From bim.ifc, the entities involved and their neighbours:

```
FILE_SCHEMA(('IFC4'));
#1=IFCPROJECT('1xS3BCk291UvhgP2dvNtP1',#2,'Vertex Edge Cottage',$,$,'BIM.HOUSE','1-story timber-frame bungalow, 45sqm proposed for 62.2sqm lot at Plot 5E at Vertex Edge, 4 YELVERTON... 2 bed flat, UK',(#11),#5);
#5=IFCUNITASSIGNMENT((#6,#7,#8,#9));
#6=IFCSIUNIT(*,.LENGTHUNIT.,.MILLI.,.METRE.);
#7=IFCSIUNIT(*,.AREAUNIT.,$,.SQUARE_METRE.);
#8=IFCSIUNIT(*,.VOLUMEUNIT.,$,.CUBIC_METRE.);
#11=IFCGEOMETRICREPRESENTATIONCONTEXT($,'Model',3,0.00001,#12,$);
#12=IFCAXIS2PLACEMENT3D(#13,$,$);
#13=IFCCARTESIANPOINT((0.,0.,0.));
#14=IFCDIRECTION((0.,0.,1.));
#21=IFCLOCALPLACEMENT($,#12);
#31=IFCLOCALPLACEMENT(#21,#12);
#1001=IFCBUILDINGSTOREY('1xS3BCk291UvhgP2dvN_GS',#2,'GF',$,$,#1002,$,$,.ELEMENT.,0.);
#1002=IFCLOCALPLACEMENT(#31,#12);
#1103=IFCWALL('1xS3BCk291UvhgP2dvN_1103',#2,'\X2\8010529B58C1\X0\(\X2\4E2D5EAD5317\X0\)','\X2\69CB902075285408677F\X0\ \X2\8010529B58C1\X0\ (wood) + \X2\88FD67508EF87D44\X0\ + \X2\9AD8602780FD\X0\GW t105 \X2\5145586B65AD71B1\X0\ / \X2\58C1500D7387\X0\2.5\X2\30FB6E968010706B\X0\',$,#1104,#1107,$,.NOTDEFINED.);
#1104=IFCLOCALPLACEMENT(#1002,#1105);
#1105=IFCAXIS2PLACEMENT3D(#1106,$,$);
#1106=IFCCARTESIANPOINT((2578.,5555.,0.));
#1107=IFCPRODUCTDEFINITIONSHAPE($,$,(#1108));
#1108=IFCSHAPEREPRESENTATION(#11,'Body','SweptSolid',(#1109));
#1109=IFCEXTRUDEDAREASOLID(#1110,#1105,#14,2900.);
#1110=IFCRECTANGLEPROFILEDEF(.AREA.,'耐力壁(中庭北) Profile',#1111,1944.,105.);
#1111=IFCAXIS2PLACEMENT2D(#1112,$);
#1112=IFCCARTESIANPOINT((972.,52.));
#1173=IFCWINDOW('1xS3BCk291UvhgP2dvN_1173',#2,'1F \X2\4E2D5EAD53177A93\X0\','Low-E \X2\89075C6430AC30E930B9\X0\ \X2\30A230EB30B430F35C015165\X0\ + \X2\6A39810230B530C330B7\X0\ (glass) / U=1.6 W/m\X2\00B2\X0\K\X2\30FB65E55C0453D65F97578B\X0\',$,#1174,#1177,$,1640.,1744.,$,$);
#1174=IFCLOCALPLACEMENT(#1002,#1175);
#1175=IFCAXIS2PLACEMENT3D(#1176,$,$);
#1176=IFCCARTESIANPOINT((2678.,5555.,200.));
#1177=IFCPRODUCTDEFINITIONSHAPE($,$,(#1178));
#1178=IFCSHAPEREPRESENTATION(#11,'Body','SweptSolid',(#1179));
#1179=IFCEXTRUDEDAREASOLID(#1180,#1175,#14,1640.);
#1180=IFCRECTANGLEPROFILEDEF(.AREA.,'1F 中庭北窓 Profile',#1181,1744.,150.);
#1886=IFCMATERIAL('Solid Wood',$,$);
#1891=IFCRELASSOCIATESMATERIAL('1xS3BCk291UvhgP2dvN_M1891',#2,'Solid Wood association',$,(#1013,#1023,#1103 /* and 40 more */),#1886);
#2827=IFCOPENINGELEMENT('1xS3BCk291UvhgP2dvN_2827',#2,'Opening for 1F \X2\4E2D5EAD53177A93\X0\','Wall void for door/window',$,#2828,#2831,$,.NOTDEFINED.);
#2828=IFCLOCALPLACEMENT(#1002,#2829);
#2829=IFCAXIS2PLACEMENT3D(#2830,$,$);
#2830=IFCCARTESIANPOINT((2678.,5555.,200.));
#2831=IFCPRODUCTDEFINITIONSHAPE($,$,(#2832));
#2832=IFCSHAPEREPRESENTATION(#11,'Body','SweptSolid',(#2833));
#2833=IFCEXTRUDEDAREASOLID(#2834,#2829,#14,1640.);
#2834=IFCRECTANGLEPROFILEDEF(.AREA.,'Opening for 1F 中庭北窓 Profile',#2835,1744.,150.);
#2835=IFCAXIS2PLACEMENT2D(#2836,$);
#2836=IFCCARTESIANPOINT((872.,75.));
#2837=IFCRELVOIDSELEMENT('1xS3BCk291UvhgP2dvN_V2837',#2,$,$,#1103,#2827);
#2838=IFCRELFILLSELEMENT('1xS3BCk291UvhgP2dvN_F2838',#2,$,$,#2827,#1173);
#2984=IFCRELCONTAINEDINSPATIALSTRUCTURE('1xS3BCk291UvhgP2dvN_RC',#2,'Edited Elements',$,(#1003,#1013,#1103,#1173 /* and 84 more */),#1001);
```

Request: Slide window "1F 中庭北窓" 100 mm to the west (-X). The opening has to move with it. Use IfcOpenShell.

```python
import ifcopenshell
import ifcopenshell.api.geometry
import ifcopenshell.util.placement
import ifcopenshell.util.unit

model = ifcopenshell.open("bim.ifc")
unit_scale = ifcopenshell.util.unit.calculate_unit_scale(model)

window = model.by_guid("1xS3BCk291UvhgP2dvN_1173")
opening = window.FillsVoids[0].RelatingOpeningElement
wall = opening.VoidsElements[0].RelatingBuildingElement

wall_matrix = ifcopenshell.util.placement.get_local_placement(wall.ObjectPlacement)
shift = wall_matrix[:3, 0] * -0.1 / unit_scale
before = ifcopenshell.util.placement.get_local_placement(window.ObjectPlacement)[:3, 3].copy()

# The window is not placed relative to its opening, so move both.
for product in (opening, window):
    matrix = ifcopenshell.util.placement.get_local_placement(product.ObjectPlacement)
    matrix[:3, 3] += shift
    ifcopenshell.api.geometry.edit_object_placement(model, product=product, matrix=matrix, is_si=False)

after = ifcopenshell.util.placement.get_local_placement(window.ObjectPlacement)[:3, 3]
print("window moved by", (after - before).round(3) + 0.0)

model.write("bim_v2.ifc")
```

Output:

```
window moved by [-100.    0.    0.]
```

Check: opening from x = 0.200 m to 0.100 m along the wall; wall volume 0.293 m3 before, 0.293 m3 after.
